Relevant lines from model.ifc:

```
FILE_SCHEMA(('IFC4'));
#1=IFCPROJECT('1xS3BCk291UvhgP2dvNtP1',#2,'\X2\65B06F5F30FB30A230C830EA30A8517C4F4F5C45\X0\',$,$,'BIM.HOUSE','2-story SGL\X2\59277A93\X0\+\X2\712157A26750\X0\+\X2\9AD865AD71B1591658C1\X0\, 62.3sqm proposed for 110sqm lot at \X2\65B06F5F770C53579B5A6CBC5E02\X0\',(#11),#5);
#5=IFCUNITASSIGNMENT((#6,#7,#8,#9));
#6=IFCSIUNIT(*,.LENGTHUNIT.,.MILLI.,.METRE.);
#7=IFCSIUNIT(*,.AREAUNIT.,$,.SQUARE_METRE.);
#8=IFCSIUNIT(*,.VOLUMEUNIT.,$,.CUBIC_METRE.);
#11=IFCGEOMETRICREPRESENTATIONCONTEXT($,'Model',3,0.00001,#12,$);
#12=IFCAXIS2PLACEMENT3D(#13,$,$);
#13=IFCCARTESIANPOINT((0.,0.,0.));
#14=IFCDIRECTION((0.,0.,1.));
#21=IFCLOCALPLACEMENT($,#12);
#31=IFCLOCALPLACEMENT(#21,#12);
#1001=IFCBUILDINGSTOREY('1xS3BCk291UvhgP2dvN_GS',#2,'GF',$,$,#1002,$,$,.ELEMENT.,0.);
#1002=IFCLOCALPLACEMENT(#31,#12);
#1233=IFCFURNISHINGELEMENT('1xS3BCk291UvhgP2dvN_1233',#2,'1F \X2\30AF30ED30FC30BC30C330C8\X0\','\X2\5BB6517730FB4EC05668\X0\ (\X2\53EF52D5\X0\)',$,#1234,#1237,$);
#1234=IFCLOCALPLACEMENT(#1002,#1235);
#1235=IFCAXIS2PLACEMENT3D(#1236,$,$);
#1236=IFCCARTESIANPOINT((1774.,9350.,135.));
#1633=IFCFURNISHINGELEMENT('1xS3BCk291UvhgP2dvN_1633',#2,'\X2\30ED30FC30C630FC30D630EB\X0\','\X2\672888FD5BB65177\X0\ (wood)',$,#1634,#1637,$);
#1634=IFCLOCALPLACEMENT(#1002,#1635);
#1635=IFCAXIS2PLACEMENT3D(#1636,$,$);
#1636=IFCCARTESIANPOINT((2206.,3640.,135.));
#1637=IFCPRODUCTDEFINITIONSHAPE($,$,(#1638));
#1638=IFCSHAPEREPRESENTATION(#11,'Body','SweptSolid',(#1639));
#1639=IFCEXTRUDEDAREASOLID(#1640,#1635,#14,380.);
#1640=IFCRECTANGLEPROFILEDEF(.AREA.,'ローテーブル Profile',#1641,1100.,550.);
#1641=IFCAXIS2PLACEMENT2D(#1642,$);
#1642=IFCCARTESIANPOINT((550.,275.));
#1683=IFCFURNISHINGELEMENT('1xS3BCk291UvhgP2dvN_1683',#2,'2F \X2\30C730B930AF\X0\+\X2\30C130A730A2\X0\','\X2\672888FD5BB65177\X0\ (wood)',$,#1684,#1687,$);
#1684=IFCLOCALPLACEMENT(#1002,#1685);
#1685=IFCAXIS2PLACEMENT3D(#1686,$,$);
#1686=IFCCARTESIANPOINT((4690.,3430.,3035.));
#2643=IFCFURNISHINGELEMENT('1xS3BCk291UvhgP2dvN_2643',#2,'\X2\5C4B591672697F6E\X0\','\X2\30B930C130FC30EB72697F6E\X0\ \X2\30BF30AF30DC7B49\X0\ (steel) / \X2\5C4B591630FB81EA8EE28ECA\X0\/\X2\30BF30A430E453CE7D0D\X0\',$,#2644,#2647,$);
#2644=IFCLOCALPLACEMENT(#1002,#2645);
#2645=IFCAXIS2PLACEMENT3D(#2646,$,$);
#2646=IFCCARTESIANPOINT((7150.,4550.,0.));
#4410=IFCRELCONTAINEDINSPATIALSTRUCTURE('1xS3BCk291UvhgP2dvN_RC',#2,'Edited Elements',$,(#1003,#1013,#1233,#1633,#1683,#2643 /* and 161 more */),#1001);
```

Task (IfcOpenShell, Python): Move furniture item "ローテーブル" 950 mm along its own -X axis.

```python
import ifcopenshell
import ifcopenshell.api.geometry
import ifcopenshell.util.placement
import ifcopenshell.util.unit

model = ifcopenshell.open("model.ifc")
unit_scale = ifcopenshell.util.unit.calculate_unit_scale(model)

item = model.by_guid("1xS3BCk291UvhgP2dvN_1633")
matrix = ifcopenshell.util.placement.get_local_placement(item.ObjectPlacement)
matrix[:3, 3] -= matrix[:3, 0] * 0.95 / unit_scale
ifcopenshell.api.geometry.edit_object_placement(model, product=item, matrix=matrix, is_si=False)

print(ifcopenshell.util.placement.get_local_placement(item.ObjectPlacement).round(3) + 0.0)

model.write("model_edited.ifc")
```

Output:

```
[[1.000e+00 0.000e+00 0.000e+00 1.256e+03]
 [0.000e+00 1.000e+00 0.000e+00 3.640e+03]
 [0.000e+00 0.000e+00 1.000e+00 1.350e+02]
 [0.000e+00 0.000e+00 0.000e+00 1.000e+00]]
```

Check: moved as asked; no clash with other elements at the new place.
